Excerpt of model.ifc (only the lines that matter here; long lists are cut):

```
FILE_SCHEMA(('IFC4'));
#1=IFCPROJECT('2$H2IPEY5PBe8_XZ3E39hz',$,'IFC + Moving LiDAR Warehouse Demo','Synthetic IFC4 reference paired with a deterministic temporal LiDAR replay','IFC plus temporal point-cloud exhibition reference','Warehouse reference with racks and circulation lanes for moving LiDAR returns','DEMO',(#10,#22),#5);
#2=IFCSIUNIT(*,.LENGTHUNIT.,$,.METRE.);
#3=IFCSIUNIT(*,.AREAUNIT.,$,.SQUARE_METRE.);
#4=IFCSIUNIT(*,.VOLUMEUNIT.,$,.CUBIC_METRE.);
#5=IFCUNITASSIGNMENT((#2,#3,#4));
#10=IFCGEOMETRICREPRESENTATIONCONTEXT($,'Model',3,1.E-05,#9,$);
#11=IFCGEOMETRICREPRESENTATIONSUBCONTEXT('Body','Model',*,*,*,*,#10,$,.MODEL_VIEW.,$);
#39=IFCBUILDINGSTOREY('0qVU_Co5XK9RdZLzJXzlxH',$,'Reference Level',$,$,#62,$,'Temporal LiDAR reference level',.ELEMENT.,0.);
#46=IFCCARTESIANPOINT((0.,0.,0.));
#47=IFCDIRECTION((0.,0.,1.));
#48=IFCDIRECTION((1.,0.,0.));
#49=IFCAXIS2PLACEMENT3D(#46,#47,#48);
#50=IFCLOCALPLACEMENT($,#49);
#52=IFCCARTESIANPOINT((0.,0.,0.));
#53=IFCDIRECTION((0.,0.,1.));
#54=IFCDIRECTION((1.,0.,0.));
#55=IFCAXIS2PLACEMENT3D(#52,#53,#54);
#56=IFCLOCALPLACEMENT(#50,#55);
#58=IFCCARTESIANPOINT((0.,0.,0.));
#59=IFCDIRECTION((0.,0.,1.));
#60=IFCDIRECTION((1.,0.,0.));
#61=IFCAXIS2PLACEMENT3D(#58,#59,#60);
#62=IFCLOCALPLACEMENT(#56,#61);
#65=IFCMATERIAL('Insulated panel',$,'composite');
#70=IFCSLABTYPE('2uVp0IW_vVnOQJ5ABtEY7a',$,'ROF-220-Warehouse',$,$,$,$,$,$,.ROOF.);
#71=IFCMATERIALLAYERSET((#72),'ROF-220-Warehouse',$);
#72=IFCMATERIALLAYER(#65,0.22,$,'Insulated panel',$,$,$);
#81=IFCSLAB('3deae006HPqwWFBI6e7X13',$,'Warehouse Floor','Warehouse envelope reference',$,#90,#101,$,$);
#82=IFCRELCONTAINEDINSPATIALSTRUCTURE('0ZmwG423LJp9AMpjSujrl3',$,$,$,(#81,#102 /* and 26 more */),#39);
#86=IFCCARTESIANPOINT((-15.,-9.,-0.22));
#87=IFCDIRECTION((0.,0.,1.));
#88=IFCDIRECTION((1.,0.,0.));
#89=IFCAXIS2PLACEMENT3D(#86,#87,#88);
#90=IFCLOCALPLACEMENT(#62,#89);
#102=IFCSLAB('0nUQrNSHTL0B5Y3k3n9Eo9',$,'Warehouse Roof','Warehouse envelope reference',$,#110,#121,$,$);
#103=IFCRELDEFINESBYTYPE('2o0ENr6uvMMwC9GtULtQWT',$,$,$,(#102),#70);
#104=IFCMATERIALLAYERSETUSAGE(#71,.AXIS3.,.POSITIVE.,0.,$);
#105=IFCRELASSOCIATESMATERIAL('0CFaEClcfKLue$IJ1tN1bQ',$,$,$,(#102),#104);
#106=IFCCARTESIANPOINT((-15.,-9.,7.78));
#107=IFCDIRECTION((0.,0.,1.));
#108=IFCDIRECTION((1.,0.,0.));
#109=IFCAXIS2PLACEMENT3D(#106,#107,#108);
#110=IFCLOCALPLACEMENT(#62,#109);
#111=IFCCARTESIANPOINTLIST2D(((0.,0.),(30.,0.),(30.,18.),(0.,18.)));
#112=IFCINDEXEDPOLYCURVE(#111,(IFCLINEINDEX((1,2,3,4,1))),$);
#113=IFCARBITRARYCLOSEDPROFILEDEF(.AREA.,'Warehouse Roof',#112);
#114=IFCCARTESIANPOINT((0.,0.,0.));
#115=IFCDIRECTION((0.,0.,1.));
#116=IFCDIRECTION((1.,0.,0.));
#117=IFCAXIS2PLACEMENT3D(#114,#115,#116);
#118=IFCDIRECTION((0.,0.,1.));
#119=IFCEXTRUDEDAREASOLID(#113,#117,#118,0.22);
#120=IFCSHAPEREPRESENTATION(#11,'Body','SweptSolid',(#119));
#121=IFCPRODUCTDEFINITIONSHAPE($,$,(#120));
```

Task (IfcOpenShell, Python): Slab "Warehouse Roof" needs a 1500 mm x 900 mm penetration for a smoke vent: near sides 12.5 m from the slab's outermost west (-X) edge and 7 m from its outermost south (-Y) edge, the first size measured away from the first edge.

```python
import numpy as np
import ifcopenshell
import ifcopenshell.api.feature
import ifcopenshell.api.geometry
import ifcopenshell.api.root
import ifcopenshell.geom
import ifcopenshell.util.placement
import ifcopenshell.util.representation
import ifcopenshell.util.shape
import ifcopenshell.util.unit

model = ifcopenshell.open("model.ifc")
unit_scale = ifcopenshell.util.unit.calculate_unit_scale(model)
settings = ifcopenshell.geom.settings()


def volume(element):
    """Net volume in cubic metres, openings subtracted."""
    shape = ifcopenshell.geom.create_shape(settings, element)
    return ifcopenshell.util.shape.get_volume(shape.geometry)


slab = model.by_guid("0nUQrNSHTL0B5Y3k3n9Eo9")
before = volume(slab)

# Extent in the slab's own axes, in metres. The edges named are its -X and -Y sides.
slab_shape = ifcopenshell.geom.create_shape(settings, slab)
vertices = ifcopenshell.util.shape.get_vertices(slab_shape.geometry)
x_min, y_min, bottom = vertices.min(axis=0)
top = vertices[:, 2].max()

opening = ifcopenshell.api.root.create_entity(model, ifc_class="IfcOpeningElement", name="Smoke vent opening", predefined_type="OPENING")
context = ifcopenshell.util.representation.get_context(model, "Model", "Body", "MODEL_VIEW")
width, depth = 1.5, 0.9
outline = [(0.0, 0.0), (width, 0.0), (width, depth), (0.0, depth), (0.0, 0.0)]
# Overshoot both faces by 50 mm so the cut is clean.
shape = ifcopenshell.api.geometry.add_slab_representation(
    model, context=context, depth=top - bottom + 0.1, polyline=outline
)
ifcopenshell.api.geometry.assign_representation(model, product=opening, representation=shape)

matrix = ifcopenshell.util.placement.get_local_placement(slab.ObjectPlacement)
matrix[:, 3] = matrix @ np.append(np.array([x_min + 12.5, y_min + 7, bottom - 0.05]) / unit_scale, 1.0)
ifcopenshell.api.geometry.edit_object_placement(model, product=opening, matrix=matrix, is_si=False)
ifcopenshell.api.feature.add_feature(model, feature=opening, element=slab)

after = volume(slab)

print(f"slab volume {before:.3f} -> {after:.3f} m3")

model.write("model_rev.ifc")
```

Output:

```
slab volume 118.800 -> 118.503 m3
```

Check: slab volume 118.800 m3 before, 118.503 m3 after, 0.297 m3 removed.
